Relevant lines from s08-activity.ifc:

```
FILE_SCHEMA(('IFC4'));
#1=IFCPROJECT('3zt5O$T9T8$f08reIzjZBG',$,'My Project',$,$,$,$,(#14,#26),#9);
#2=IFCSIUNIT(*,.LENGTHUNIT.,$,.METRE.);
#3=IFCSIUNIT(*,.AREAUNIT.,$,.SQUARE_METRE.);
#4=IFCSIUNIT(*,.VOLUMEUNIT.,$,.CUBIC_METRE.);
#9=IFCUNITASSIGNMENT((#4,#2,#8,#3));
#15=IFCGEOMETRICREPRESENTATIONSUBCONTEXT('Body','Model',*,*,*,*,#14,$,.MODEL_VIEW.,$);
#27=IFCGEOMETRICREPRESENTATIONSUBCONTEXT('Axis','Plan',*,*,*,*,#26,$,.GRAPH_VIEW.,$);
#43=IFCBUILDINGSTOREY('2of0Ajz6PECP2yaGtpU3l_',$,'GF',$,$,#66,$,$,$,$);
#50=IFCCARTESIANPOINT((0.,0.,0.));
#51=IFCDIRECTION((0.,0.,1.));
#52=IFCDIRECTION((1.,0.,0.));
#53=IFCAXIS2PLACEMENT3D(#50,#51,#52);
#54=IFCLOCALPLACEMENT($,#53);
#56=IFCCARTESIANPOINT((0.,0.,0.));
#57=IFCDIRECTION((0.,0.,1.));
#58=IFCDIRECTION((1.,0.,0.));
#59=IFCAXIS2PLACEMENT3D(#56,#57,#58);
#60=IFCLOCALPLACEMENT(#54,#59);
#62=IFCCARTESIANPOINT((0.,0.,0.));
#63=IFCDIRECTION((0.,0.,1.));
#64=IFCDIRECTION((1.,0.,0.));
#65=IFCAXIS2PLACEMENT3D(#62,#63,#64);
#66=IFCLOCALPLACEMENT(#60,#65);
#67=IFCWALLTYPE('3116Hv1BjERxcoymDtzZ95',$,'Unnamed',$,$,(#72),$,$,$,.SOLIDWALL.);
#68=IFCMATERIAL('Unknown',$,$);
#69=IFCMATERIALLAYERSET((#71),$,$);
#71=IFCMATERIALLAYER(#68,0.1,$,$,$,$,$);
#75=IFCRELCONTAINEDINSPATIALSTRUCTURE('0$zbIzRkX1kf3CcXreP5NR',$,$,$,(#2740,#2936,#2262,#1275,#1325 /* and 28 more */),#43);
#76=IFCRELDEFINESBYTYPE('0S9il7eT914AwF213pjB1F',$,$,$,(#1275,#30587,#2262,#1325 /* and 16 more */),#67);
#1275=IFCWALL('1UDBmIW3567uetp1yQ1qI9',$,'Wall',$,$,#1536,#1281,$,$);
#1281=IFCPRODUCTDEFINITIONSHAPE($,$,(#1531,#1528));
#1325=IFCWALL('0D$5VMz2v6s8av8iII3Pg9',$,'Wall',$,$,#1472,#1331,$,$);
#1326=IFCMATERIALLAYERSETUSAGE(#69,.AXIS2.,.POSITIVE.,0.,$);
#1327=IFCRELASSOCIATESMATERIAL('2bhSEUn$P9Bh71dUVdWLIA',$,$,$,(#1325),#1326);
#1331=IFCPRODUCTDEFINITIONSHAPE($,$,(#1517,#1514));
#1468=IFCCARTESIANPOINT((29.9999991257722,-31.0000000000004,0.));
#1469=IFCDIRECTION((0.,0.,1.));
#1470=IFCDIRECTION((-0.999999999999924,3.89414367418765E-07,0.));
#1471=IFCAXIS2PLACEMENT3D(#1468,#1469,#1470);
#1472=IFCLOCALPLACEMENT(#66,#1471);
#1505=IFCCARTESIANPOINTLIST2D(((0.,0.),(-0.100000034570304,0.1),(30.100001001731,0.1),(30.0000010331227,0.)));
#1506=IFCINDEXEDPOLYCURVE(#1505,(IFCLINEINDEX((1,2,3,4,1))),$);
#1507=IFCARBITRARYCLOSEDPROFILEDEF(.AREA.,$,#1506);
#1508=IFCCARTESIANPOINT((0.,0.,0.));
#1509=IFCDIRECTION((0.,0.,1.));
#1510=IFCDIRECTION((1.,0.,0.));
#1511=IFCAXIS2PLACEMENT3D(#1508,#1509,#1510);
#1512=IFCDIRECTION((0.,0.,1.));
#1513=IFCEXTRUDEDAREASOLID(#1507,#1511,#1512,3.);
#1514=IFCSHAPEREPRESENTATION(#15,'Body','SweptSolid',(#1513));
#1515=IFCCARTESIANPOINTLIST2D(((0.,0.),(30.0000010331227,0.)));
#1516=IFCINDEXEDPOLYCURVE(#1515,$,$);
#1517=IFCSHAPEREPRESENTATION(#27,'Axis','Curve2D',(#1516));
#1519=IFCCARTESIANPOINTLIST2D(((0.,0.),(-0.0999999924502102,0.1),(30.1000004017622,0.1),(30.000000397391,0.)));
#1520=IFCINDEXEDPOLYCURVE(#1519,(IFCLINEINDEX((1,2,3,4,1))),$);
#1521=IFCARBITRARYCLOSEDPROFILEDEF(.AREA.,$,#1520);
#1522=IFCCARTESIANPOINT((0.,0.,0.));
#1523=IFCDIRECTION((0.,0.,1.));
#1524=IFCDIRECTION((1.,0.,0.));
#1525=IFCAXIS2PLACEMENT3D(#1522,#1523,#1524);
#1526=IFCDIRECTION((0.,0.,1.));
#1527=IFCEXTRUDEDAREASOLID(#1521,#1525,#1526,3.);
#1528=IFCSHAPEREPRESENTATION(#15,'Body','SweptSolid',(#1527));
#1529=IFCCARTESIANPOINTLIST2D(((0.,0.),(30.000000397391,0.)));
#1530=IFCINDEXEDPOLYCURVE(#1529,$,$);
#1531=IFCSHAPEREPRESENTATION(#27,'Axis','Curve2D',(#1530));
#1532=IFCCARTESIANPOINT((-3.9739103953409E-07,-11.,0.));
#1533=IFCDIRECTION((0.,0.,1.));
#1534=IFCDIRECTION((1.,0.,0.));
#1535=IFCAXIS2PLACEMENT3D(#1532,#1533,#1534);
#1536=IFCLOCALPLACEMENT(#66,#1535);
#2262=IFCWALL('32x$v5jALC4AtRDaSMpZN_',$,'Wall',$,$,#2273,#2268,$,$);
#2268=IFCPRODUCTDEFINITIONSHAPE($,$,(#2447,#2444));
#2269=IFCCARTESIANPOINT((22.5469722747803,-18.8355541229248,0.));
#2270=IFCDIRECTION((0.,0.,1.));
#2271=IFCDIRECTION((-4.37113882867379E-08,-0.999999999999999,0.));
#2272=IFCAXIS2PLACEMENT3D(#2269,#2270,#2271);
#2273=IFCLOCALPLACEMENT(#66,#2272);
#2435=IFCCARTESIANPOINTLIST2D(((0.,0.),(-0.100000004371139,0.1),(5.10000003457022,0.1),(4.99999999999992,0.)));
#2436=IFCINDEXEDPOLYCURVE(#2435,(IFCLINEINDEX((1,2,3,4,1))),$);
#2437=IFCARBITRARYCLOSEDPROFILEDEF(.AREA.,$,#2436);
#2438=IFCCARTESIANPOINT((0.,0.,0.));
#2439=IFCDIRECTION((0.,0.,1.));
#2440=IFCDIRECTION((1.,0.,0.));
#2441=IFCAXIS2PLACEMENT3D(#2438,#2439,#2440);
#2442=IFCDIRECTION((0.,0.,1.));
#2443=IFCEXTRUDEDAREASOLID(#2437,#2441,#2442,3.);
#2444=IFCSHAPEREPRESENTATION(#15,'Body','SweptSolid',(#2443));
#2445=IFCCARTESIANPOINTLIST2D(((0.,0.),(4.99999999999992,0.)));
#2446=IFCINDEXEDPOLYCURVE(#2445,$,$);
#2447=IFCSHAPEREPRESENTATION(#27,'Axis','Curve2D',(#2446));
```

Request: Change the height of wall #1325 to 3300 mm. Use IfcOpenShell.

```python
import ifcopenshell
import ifcopenshell.geom
import ifcopenshell.util.representation
import ifcopenshell.util.shape

model = ifcopenshell.open("s08-activity.ifc")
settings = ifcopenshell.geom.settings()


def volume(element):
    """Net volume in cubic metres, openings subtracted."""
    shape = ifcopenshell.geom.create_shape(settings, element)
    return ifcopenshell.util.shape.get_volume(shape.geometry)


wall = model.by_guid("0D$5VMz2v6s8av8iII3Pg9")
before = volume(wall)

body = ifcopenshell.util.representation.get_representation(wall, "Model", "Body")
solid = body.Items[0]
old_height = solid.Depth
solid.Depth = 3.3
after = volume(wall)

print(f"height {old_height:g} -> {solid.Depth:g}, volume {before:.3f} -> {after:.3f} m3")

model.write("s08-activity_edited.ifc")
```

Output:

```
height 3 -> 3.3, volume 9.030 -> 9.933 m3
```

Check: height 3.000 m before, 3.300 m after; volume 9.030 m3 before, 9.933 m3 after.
